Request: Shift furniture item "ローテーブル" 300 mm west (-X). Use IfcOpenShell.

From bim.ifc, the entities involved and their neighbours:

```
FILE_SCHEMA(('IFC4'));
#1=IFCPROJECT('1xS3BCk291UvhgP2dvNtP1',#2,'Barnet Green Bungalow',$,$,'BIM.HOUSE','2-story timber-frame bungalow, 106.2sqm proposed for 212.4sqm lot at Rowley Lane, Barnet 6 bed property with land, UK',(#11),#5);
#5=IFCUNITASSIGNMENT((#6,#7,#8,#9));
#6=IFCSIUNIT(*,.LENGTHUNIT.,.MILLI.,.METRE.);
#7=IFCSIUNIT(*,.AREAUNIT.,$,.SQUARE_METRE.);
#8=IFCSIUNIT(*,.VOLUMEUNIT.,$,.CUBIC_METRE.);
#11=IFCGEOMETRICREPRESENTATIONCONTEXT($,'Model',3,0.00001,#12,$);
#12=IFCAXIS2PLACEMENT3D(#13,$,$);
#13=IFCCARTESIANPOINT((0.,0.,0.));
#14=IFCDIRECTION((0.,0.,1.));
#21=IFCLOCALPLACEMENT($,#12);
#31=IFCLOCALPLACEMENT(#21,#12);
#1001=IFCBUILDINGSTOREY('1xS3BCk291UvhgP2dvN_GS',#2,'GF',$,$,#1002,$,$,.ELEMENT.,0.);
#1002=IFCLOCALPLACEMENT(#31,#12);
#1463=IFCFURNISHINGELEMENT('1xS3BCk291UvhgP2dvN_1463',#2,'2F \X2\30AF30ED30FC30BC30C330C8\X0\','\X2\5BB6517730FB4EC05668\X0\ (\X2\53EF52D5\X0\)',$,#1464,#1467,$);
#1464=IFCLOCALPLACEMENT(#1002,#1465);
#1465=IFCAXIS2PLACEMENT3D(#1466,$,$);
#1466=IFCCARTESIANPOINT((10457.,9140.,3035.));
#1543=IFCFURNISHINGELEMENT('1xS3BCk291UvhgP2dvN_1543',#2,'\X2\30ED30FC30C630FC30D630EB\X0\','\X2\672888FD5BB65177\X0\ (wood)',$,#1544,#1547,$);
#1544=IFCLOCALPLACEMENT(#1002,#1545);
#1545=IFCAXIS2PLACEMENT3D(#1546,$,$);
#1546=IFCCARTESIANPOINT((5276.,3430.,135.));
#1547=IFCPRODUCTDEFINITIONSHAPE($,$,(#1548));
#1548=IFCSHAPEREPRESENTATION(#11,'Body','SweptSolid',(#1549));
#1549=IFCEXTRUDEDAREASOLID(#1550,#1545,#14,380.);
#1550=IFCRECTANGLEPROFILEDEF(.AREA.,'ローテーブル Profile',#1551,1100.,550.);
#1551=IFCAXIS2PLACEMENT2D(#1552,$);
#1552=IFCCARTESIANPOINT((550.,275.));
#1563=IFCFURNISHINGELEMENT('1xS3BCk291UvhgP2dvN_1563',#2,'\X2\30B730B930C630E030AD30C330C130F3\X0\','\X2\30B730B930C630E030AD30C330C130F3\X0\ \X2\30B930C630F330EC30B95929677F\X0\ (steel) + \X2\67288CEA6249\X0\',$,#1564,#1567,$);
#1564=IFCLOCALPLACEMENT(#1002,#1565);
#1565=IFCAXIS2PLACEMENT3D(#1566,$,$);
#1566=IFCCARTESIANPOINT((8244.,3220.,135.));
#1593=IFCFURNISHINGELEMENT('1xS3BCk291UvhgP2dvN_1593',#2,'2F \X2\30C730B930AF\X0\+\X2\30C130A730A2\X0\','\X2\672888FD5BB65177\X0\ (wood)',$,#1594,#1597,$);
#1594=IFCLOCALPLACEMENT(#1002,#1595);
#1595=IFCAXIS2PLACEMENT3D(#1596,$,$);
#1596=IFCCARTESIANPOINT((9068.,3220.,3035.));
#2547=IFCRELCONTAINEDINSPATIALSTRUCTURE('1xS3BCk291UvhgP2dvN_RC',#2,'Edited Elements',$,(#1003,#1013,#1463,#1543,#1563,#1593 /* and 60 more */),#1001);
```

```python
import ifcopenshell
import ifcopenshell.api.geometry
import ifcopenshell.util.placement

model = ifcopenshell.open("bim.ifc")

item = model.by_id(1543)
matrix = ifcopenshell.util.placement.get_local_placement(item.ObjectPlacement)
matrix[0, 3] -= 300.0
ifcopenshell.api.geometry.edit_object_placement(model, product=item, matrix=matrix, is_si=False)

print(ifcopenshell.util.placement.get_local_placement(item.ObjectPlacement).round(3) + 0.0)

model.write("bim-out.ifc")
```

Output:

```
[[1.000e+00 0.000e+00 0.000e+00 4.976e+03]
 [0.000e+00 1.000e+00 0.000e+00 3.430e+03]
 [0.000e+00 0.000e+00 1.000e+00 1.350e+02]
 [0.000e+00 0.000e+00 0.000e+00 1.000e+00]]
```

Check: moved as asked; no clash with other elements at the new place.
